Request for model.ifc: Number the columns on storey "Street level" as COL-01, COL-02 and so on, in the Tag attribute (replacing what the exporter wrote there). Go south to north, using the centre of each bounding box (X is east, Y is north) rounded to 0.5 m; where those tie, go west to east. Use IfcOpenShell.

First a look at what the model holds.

```python
import ifcopenshell
import ifcopenshell.util.element
import ifcopenshell.util.placement

model = ifcopenshell.open("model.ifc")
print(model.schema)
storey = next(s for s in model.by_type("IfcBuildingStorey") if s.Name == "Street level")
columns = [e for e in ifcopenshell.util.element.get_decomposition(storey) if e.is_a("IfcColumn")]
for e in sorted(columns, key=lambda e: e.id()):
    origin = ifcopenshell.util.placement.get_local_placement(e.ObjectPlacement)[:3, 3]
    print(e.id(), e.Tag, e.Name, origin.round(2) + 0.0, sep=" | ")
```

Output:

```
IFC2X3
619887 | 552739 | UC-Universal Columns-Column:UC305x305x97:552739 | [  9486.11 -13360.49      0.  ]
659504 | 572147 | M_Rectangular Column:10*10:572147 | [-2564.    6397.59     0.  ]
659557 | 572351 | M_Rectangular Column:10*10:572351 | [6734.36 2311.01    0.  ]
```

```python
import ifcopenshell
import ifcopenshell.geom
import ifcopenshell.util.element
import ifcopenshell.util.shape

model = ifcopenshell.open("model.ifc")
settings = ifcopenshell.geom.settings()
settings.set("use-world-coords", True)


def centre(element):
    shape = ifcopenshell.geom.create_shape(settings, element)
    return ifcopenshell.util.shape.get_bbox_centroid(shape.geometry)


storey = next(s for s in model.by_type("IfcBuildingStorey") if s.Name == "Street level")
columns = [e for e in ifcopenshell.util.element.get_decomposition(storey) if e.is_a("IfcColumn")]

# Insertion points can sit at a corner or the storey origin, so sort by the geometry (in metres).
centres = {e: centre(e) for e in columns}
columns.sort(key=lambda e: (round(centres[e][1] / 0.5), centres[e][0]))

for i, e in enumerate(columns, start=1):
    number = f"COL-{i:02d}"
    e.Tag = number
    print(e.id(), number)

model.write("model_v2.ifc")
```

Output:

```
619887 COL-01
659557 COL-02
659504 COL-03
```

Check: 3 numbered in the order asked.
